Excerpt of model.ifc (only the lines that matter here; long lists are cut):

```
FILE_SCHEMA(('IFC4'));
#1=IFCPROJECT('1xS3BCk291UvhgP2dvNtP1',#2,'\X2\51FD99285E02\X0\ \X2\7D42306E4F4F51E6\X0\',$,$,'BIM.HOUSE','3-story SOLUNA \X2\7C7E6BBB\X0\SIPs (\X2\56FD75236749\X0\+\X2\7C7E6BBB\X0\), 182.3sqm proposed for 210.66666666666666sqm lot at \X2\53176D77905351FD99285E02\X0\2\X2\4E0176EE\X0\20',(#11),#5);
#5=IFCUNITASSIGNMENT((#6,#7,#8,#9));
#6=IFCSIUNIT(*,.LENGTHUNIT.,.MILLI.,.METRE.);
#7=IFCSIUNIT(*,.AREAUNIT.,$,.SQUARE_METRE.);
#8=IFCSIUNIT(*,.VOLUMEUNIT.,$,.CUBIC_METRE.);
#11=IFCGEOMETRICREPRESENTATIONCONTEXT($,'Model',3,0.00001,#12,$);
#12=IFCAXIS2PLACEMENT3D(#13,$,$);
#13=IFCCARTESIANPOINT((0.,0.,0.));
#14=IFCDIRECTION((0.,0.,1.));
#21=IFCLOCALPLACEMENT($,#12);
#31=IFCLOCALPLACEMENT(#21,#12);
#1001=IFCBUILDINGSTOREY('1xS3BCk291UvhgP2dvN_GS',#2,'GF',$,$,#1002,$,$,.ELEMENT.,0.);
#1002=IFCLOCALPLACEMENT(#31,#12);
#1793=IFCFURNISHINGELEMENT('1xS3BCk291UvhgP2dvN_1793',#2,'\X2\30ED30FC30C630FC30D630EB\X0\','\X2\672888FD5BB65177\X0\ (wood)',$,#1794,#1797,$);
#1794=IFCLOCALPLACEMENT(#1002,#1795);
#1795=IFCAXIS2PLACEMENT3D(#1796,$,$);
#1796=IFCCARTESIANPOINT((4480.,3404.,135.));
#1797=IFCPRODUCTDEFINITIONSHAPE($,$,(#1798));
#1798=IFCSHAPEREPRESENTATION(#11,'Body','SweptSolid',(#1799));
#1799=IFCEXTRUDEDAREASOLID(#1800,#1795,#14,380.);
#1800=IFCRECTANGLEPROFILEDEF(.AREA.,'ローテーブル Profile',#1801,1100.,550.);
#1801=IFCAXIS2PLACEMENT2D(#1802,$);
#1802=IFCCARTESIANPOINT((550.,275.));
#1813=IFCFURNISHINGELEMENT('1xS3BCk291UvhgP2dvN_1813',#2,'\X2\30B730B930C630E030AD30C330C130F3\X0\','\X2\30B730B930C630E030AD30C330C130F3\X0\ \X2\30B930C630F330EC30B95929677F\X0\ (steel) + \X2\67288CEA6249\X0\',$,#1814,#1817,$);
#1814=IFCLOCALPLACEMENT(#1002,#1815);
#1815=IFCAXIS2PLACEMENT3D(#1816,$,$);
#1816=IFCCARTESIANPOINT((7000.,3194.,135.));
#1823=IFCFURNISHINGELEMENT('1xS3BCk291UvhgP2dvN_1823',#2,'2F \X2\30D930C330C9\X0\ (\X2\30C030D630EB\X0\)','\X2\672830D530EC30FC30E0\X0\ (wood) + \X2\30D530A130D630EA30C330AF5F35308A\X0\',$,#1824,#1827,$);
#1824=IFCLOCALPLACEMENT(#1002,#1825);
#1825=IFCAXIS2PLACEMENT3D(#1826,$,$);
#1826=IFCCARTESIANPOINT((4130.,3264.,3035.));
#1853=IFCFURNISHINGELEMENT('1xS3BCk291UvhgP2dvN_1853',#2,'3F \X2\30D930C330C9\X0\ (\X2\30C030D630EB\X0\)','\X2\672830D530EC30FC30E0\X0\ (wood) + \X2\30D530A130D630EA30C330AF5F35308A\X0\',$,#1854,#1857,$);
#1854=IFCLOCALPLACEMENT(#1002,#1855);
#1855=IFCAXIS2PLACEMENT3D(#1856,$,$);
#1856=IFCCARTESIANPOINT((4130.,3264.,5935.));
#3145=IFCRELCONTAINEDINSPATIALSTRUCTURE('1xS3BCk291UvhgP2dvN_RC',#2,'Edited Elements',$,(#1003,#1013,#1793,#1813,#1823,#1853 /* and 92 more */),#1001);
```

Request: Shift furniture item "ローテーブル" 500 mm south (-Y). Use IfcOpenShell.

```python
import ifcopenshell
import ifcopenshell.api.geometry
import ifcopenshell.util.placement
import ifcopenshell.util.unit

model = ifcopenshell.open("model.ifc")
unit_scale = ifcopenshell.util.unit.calculate_unit_scale(model)

item = model.by_guid("1xS3BCk291UvhgP2dvN_1793")
matrix = ifcopenshell.util.placement.get_local_placement(item.ObjectPlacement)
matrix[1, 3] -= 0.5 / unit_scale
ifcopenshell.api.geometry.edit_object_placement(model, product=item, matrix=matrix, is_si=False)

print(ifcopenshell.util.placement.get_local_placement(item.ObjectPlacement).round(3) + 0.0)

model.write("model-out.ifc")
```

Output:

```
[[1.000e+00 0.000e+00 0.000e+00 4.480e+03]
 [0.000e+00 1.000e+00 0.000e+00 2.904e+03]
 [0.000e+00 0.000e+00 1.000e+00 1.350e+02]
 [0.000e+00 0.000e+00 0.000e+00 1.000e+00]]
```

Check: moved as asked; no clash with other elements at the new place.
